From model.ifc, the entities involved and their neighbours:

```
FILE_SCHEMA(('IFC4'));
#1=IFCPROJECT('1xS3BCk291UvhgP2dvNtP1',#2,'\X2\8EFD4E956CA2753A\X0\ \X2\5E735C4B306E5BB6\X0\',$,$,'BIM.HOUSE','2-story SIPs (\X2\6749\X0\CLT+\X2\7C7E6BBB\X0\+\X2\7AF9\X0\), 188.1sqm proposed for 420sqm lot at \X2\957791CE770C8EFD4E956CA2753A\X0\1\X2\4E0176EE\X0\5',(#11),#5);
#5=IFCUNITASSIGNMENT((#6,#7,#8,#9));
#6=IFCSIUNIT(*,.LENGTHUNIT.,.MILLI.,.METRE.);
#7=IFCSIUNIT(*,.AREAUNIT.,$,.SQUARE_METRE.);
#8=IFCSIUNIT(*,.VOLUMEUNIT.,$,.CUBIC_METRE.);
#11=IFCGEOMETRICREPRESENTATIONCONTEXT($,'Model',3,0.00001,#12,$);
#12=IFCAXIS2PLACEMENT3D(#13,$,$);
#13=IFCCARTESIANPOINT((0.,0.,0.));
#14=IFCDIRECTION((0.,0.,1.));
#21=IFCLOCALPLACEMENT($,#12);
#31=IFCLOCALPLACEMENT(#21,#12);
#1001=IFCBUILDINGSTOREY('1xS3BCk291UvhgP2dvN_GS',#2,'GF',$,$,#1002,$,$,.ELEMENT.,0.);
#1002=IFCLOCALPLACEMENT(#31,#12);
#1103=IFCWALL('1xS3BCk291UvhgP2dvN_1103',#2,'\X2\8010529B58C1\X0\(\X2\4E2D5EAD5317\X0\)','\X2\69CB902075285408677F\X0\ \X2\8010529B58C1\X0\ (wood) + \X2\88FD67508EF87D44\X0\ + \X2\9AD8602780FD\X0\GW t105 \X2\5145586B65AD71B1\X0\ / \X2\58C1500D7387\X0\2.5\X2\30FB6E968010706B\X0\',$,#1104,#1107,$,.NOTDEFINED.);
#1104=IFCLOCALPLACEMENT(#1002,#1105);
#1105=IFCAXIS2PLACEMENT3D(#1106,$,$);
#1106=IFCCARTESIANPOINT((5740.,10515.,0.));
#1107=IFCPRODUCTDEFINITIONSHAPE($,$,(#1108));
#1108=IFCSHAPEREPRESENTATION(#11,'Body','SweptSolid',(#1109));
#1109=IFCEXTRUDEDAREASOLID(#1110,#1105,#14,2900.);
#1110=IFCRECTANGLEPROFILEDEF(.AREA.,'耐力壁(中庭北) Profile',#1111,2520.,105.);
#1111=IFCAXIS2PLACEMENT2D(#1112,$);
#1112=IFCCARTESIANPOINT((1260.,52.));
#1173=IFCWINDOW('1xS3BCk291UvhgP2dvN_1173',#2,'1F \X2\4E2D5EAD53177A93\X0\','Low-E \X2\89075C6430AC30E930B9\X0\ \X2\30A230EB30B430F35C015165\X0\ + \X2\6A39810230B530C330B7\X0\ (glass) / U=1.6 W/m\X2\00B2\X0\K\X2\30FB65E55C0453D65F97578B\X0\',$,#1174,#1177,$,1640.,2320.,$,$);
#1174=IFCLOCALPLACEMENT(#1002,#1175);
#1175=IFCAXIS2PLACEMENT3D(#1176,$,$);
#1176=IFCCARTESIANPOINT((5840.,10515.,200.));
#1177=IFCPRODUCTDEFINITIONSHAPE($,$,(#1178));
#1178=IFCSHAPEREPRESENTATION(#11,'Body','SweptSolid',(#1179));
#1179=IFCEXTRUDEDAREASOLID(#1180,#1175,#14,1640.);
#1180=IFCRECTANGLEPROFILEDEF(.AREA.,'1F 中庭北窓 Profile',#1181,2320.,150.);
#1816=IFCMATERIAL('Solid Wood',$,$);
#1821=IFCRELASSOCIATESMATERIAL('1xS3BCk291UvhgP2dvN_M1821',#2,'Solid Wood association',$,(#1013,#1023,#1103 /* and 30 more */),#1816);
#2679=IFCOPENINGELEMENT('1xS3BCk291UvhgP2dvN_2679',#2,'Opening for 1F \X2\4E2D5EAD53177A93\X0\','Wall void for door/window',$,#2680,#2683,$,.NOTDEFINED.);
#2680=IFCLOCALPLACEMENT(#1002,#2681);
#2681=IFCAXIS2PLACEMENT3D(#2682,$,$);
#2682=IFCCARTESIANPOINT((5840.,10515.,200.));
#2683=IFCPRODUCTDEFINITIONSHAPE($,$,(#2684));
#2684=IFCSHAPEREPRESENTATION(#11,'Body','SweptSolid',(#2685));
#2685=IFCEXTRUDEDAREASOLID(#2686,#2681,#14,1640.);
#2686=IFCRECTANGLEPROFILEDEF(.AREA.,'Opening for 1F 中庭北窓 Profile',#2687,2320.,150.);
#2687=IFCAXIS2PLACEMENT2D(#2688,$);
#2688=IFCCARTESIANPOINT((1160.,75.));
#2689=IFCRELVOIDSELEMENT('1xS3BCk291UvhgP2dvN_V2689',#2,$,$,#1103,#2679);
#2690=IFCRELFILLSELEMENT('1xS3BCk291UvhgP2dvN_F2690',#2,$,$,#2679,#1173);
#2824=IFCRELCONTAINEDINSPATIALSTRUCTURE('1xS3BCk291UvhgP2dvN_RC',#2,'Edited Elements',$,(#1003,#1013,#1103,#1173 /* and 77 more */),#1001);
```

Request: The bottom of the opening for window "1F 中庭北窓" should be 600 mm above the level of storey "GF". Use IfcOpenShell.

```python
import numpy as np
import ifcopenshell
import ifcopenshell.api.geometry
import ifcopenshell.geom
import ifcopenshell.util.element
import ifcopenshell.util.placement
import ifcopenshell.util.shape
import ifcopenshell.util.unit

model = ifcopenshell.open("model.ifc")
unit_scale = ifcopenshell.util.unit.calculate_unit_scale(model)

window = model.by_guid("1xS3BCk291UvhgP2dvN_1173")
opening = window.FillsVoids[0].RelatingOpeningElement
storey = ifcopenshell.util.element.get_container(window, ifc_class="IfcBuildingStorey")
level = ifcopenshell.util.placement.get_local_placement(storey.ObjectPlacement)[2, 3]

# The opening's origin need not be at the sill, so measure its lowest point.
shape = ifcopenshell.geom.create_shape(ifcopenshell.geom.settings(), opening)
bottom = ifcopenshell.util.shape.get_shape_bottom_elevation(shape, shape.geometry) / unit_scale
dz = level + 600.0 - bottom

shift = np.array([0.0, 0.0, dz])
# The window is not placed relative to its opening, so move both.
for product in (opening, window):
    matrix = ifcopenshell.util.placement.get_local_placement(product.ObjectPlacement)
    matrix[:3, 3] += shift
    ifcopenshell.api.geometry.edit_object_placement(model, product=product, matrix=matrix, is_si=False)

print(f"moved by {dz * unit_scale:+.3f} m")

model.write("model_v2.ifc")
```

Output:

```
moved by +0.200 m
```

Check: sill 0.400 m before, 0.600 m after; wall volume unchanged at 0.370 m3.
